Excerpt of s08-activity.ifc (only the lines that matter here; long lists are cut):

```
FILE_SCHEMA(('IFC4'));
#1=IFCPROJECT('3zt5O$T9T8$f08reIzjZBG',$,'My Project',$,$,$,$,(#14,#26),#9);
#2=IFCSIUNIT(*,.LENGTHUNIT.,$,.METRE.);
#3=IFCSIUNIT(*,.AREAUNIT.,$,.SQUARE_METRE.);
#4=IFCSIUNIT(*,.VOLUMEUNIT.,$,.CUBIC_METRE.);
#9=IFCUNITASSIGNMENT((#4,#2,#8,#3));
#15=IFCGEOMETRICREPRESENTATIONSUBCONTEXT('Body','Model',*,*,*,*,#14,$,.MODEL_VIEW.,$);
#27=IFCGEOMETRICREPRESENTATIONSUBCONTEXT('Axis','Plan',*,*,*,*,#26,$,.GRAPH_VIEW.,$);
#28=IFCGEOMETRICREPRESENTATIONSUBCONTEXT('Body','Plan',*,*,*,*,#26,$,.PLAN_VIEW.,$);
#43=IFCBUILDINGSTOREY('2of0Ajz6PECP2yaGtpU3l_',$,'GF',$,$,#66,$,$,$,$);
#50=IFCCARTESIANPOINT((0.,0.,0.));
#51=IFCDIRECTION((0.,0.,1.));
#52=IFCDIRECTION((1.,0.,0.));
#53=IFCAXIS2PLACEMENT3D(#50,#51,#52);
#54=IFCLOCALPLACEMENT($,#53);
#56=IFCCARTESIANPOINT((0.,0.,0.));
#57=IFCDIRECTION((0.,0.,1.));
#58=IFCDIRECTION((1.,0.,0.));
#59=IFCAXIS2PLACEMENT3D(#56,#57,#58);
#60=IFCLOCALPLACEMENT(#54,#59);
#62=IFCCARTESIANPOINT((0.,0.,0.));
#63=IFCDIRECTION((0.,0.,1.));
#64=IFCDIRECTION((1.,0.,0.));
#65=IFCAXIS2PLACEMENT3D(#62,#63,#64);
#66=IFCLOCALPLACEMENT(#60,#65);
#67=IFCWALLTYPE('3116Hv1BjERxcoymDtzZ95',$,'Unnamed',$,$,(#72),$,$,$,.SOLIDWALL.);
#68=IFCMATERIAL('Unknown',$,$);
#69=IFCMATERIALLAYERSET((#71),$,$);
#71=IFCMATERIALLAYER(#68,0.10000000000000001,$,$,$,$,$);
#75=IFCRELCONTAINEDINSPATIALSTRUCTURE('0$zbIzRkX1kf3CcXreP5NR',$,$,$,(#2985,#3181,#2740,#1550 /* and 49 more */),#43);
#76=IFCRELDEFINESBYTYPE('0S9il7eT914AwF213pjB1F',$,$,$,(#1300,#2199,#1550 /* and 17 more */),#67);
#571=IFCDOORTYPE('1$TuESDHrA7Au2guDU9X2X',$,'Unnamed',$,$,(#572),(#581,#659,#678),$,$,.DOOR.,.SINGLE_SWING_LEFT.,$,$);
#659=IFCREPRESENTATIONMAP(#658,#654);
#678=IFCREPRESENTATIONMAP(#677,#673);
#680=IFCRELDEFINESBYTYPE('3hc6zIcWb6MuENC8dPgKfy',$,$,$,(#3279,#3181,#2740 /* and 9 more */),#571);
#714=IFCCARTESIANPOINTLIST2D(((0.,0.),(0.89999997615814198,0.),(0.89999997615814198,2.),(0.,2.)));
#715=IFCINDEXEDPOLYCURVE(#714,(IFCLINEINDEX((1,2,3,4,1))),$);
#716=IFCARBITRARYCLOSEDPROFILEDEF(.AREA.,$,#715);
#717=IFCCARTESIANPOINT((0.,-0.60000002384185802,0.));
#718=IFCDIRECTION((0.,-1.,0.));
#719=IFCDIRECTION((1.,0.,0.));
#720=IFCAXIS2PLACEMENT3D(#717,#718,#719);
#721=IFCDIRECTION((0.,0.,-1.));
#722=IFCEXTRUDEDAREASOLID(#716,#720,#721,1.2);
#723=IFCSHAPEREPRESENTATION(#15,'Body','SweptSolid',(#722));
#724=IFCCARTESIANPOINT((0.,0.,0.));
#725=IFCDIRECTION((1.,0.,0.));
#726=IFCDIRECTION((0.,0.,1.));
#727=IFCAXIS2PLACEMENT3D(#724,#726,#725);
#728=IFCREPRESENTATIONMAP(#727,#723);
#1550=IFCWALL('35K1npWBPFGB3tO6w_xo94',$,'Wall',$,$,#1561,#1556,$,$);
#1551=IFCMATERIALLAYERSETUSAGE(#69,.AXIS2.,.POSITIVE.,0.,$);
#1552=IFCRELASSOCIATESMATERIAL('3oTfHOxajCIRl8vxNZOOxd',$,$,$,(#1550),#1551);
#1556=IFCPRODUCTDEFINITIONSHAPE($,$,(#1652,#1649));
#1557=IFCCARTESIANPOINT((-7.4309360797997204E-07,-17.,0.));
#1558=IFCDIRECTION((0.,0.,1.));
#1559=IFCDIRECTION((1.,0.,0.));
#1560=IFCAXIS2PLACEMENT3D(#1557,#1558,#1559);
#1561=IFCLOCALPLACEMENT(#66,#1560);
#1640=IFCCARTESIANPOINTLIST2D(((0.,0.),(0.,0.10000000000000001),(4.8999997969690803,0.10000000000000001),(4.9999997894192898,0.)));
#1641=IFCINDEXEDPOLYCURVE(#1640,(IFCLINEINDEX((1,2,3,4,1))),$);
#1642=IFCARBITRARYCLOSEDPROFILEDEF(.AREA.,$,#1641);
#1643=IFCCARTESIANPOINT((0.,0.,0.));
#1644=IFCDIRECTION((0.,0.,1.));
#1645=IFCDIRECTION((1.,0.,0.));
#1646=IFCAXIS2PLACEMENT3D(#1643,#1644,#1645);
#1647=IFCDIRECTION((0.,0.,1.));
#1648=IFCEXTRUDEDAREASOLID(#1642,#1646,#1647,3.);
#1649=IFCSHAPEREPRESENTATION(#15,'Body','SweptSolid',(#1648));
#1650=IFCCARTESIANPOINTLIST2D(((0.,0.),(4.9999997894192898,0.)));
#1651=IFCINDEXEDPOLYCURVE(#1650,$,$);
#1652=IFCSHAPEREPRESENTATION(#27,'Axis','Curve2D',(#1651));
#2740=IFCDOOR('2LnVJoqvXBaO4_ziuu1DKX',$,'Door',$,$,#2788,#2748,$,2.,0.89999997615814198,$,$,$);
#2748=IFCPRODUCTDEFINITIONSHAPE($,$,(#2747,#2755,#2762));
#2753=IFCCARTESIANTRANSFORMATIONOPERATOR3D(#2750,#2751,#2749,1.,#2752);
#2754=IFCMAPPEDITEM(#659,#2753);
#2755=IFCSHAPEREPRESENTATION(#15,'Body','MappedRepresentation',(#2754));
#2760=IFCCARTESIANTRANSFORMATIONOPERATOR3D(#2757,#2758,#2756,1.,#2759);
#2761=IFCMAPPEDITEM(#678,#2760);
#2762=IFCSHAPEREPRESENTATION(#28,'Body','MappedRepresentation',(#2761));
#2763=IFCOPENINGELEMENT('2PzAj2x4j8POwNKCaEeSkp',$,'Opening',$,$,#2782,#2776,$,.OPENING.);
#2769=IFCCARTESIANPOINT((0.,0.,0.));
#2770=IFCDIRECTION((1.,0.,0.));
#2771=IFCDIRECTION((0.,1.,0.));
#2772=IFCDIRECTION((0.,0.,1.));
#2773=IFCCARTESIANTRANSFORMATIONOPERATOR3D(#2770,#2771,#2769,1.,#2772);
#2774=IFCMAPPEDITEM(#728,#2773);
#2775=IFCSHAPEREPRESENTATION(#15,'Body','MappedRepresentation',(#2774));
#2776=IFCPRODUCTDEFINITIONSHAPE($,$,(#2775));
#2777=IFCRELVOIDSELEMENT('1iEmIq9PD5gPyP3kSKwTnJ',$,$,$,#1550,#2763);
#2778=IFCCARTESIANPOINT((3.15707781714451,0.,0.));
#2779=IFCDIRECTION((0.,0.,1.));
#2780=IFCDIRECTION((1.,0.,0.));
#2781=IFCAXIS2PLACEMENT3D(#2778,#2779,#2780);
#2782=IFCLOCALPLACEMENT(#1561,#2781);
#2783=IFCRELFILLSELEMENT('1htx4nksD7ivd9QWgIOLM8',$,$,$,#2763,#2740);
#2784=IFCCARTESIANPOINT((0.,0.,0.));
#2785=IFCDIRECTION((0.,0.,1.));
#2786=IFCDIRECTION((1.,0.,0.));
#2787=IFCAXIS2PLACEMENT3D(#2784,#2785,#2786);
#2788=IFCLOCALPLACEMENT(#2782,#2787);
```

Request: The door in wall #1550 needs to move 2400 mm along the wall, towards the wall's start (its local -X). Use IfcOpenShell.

```python
import ifcopenshell
import ifcopenshell.api.geometry
import ifcopenshell.util.placement

model = ifcopenshell.open("s08-activity.ifc")

door = model.by_guid("2LnVJoqvXBaO4_ziuu1DKX")
opening = door.FillsVoids[0].RelatingOpeningElement
wall = opening.VoidsElements[0].RelatingBuildingElement

wall_matrix = ifcopenshell.util.placement.get_local_placement(wall.ObjectPlacement)
shift = wall_matrix[:3, 0] * -2.4
before = ifcopenshell.util.placement.get_local_placement(door.ObjectPlacement)[:3, 3].copy()

# The door is placed relative to its opening, so it follows when the opening moves.
matrix = ifcopenshell.util.placement.get_local_placement(opening.ObjectPlacement)
matrix[:3, 3] += shift
ifcopenshell.api.geometry.edit_object_placement(
    model, product=opening, matrix=matrix, is_si=False, should_transform_children=True
)

after = ifcopenshell.util.placement.get_local_placement(door.ObjectPlacement)[:3, 3]
print("door moved by", (after - before).round(3) + 0.0)

model.write("s08-activity_rev.ifc")
```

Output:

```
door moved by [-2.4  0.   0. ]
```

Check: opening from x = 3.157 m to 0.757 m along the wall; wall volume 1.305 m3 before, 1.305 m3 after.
